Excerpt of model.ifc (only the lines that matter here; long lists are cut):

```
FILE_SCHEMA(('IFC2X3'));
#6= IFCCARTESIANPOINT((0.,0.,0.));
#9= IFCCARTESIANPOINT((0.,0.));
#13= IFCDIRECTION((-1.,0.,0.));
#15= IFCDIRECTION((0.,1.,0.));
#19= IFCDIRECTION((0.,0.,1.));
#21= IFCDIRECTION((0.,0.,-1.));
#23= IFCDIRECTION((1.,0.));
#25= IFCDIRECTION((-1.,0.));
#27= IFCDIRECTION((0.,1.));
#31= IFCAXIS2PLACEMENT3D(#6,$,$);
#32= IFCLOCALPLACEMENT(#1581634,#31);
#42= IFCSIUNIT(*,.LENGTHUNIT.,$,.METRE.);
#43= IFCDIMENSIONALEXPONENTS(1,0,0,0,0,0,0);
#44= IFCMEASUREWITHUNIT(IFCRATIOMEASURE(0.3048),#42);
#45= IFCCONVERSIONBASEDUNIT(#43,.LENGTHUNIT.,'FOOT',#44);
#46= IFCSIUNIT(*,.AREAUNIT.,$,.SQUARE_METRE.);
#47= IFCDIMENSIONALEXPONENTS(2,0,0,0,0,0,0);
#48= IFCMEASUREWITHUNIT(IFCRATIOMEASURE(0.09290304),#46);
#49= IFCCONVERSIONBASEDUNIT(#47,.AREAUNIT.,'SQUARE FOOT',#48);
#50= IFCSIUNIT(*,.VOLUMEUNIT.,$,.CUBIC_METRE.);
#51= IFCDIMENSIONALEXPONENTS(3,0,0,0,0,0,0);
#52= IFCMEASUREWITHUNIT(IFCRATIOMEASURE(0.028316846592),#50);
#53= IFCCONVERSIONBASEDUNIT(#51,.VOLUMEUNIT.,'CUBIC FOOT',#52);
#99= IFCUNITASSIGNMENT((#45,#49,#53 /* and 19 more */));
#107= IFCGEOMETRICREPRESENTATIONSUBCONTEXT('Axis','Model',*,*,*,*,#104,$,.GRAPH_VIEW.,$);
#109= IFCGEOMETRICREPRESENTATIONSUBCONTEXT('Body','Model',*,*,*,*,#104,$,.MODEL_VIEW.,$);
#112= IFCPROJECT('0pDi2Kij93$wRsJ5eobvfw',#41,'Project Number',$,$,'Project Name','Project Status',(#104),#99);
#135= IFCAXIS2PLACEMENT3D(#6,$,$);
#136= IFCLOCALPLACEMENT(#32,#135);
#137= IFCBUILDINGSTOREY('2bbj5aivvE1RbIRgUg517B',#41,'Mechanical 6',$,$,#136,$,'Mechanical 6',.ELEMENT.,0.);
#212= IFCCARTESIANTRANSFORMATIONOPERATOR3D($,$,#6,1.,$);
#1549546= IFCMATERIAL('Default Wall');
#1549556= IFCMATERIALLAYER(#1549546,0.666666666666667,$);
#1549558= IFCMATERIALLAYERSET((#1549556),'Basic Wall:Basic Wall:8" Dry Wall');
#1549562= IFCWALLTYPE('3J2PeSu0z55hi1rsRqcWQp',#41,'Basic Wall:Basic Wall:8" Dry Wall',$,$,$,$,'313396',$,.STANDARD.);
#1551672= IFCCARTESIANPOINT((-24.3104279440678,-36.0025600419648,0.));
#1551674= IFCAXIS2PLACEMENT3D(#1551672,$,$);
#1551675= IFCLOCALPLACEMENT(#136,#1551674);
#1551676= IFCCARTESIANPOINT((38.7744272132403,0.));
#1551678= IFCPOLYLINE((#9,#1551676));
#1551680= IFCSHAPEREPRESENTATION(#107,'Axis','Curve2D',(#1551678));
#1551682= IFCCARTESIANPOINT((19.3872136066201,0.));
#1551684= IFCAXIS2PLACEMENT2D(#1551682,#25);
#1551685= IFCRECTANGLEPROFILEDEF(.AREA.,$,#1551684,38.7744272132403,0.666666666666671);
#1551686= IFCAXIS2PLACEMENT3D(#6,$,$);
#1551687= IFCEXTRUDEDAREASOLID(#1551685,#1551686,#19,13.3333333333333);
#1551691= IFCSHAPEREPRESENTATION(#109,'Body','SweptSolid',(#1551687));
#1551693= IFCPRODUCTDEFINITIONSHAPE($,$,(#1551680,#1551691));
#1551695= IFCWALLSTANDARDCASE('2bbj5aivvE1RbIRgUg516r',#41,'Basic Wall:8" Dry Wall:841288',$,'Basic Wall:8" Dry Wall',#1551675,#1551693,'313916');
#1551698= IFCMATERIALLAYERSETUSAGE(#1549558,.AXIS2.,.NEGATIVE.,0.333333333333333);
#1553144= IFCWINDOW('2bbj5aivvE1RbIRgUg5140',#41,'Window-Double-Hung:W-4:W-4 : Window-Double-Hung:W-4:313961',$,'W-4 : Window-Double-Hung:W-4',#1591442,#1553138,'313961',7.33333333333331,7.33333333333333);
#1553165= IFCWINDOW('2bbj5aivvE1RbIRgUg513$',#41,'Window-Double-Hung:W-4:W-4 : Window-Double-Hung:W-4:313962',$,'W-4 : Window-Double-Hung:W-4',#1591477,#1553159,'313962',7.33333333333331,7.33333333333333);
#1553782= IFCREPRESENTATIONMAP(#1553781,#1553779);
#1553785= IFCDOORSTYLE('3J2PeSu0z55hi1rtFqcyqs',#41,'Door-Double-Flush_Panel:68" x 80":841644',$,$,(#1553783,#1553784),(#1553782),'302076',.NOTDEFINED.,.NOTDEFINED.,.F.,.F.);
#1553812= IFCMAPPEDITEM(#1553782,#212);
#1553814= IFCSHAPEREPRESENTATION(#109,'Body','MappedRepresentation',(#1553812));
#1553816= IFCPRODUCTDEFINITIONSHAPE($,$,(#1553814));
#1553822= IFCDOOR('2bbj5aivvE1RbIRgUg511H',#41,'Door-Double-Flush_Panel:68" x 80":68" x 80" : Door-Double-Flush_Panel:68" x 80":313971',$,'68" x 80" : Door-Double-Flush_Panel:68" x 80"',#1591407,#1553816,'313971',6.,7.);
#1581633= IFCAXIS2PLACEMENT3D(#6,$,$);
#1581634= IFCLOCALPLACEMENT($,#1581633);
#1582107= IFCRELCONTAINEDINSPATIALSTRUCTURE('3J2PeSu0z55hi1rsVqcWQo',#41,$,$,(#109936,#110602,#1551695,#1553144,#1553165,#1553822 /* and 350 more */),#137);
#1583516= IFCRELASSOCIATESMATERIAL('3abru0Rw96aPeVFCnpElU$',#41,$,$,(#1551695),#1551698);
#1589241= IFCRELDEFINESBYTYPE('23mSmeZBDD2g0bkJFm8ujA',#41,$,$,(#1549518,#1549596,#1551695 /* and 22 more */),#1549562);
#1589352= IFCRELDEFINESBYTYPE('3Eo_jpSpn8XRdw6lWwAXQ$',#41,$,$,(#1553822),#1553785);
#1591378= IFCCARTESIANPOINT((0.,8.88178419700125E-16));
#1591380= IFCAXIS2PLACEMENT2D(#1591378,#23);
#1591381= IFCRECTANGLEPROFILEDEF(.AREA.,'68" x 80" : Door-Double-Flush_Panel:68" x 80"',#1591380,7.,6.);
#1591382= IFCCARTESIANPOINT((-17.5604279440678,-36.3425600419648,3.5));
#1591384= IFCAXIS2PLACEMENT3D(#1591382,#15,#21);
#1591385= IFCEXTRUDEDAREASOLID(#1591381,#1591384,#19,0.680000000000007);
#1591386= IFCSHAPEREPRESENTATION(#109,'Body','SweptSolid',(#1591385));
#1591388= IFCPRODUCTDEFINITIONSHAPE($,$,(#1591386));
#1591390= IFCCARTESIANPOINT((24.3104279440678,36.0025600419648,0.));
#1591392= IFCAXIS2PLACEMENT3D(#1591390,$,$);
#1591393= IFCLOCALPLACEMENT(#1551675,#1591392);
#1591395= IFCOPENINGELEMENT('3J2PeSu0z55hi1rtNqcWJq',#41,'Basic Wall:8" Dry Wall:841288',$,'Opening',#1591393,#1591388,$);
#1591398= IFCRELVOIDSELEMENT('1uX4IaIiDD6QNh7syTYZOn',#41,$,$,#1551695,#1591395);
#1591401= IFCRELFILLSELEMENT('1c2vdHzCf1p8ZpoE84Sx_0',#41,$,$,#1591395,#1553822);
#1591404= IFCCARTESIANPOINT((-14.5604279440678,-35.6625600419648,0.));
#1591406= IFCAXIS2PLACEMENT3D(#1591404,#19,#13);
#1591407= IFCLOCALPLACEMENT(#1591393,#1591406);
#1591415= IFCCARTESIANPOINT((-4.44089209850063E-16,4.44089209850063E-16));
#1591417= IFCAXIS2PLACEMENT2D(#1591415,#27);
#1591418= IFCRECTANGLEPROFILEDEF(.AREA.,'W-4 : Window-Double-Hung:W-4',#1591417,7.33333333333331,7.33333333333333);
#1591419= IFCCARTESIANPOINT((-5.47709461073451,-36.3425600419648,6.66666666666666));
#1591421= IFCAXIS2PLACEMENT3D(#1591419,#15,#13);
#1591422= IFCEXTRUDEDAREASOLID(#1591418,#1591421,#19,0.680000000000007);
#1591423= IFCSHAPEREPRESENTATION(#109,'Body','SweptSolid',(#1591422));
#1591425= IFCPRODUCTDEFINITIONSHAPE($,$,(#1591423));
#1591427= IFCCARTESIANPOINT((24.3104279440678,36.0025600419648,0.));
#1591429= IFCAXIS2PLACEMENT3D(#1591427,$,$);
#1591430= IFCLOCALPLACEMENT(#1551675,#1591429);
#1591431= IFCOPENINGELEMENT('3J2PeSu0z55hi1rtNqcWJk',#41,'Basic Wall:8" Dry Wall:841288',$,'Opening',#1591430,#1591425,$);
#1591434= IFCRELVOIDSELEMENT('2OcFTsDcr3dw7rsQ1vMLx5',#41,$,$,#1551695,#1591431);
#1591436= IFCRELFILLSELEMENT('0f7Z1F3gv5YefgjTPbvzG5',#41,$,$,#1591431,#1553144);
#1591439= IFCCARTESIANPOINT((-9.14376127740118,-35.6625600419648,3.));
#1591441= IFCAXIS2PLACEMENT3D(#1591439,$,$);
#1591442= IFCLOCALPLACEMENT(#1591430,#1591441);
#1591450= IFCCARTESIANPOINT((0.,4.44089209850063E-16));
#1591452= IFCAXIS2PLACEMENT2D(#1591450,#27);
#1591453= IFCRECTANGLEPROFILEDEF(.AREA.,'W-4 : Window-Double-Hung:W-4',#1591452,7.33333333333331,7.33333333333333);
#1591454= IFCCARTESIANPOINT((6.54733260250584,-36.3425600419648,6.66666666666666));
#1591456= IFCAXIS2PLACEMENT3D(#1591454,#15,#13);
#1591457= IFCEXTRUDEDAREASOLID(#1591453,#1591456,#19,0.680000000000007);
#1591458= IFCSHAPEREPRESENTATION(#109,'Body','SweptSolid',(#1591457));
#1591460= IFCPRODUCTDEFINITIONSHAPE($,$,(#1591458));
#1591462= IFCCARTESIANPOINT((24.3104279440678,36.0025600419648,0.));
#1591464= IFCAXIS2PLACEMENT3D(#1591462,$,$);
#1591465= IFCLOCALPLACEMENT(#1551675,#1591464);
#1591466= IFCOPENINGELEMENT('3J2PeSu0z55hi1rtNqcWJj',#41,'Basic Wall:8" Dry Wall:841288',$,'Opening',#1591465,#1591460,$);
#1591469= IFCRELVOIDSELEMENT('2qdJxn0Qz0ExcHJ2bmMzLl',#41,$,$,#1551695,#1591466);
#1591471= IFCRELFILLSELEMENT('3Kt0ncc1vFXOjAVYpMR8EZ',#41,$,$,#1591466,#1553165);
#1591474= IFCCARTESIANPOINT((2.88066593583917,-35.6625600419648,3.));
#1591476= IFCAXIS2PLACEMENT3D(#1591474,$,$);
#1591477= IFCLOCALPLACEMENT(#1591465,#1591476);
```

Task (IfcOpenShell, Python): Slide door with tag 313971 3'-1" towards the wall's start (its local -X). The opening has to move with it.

```python
import ifcopenshell
import ifcopenshell.api.geometry
import ifcopenshell.util.placement
import ifcopenshell.util.unit

model = ifcopenshell.open("model.ifc")
unit_scale = ifcopenshell.util.unit.calculate_unit_scale(model)

door = model.by_guid("2bbj5aivvE1RbIRgUg511H")
opening = door.FillsVoids[0].RelatingOpeningElement
wall = opening.VoidsElements[0].RelatingBuildingElement

wall_matrix = ifcopenshell.util.placement.get_local_placement(wall.ObjectPlacement)
shift = wall_matrix[:3, 0] * -37 * 0.0254 / unit_scale
before = ifcopenshell.util.placement.get_local_placement(door.ObjectPlacement)[:3, 3].copy()

# The door is placed relative to its opening, so it follows when the opening moves.
matrix = ifcopenshell.util.placement.get_local_placement(opening.ObjectPlacement)
matrix[:3, 3] += shift
ifcopenshell.api.geometry.edit_object_placement(
    model, product=opening, matrix=matrix, is_si=False, should_transform_children=True
)

after = ifcopenshell.util.placement.get_local_placement(door.ObjectPlacement)[:3, 3]
print("door moved by", (after - before).round(3) + 0.0)

model.write("model_rev.ifc")
```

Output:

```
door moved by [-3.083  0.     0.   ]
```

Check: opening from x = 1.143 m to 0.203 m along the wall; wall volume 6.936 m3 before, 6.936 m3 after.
